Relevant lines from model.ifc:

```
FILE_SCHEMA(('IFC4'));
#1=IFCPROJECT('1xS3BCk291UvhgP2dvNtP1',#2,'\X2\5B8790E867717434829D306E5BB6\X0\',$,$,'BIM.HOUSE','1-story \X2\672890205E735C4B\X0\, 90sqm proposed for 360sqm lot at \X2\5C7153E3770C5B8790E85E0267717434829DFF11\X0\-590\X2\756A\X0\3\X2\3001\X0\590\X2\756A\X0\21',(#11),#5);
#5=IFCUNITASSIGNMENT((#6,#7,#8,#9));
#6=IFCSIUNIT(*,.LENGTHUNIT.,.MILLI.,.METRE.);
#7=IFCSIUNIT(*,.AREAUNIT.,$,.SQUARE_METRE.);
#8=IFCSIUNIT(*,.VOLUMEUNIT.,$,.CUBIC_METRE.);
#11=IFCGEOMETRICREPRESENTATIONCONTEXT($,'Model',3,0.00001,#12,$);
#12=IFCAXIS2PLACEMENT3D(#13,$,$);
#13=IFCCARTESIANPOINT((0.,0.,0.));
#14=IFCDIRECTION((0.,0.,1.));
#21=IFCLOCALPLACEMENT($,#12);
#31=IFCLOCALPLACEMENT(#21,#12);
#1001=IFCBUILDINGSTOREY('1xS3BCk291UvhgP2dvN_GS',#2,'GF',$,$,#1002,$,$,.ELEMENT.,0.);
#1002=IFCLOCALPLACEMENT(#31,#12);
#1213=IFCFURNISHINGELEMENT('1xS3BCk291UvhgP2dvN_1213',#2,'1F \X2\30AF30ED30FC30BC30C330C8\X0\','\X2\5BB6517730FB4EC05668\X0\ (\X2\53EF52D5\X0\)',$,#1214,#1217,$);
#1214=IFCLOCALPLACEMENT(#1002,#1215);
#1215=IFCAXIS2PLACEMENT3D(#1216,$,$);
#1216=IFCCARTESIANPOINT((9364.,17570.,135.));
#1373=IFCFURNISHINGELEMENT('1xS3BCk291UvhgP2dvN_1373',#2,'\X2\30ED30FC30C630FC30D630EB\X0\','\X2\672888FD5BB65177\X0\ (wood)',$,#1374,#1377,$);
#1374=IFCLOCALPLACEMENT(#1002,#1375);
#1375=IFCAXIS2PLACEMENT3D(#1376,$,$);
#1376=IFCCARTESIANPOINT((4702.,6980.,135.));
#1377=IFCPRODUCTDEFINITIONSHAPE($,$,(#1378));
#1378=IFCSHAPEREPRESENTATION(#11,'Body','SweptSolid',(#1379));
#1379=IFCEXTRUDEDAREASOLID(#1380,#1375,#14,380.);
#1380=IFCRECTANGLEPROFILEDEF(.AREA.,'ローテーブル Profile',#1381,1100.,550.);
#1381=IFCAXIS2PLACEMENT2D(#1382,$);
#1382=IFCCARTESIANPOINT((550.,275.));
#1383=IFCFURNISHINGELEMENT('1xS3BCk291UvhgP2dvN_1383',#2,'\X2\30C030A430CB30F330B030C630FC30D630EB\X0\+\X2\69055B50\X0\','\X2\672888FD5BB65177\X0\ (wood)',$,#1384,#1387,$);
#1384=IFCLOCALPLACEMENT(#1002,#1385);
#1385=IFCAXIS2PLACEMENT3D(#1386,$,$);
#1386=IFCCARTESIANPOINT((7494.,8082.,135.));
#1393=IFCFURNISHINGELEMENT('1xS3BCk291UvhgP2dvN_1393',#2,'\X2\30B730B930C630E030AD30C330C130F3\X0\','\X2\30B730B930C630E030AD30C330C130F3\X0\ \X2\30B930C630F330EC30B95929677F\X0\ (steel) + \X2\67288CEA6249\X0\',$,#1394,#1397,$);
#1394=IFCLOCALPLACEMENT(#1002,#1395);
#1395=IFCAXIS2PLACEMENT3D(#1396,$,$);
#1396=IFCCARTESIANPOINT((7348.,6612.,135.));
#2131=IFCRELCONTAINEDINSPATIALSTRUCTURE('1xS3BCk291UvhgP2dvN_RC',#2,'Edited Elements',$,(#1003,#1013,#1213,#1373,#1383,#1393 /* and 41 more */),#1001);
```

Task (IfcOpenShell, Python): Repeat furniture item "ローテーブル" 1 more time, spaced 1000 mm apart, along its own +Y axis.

```python
import ifcopenshell
import ifcopenshell.api.geometry
import ifcopenshell.api.root
import ifcopenshell.util.element
import ifcopenshell.util.placement
import ifcopenshell.util.unit

model = ifcopenshell.open("model.ifc")
unit_scale = ifcopenshell.util.unit.calculate_unit_scale(model)


def reuse_history(source, copy):
    """copy_class also copies each property set's owner history, people and application; keep the originals."""
    for rel in copy.IsDefinedBy:
        if rel.is_a("IfcRelDefinesByProperties") and (history := rel.RelatingPropertyDefinition.OwnerHistory):
            rel.RelatingPropertyDefinition.OwnerHistory = source.OwnerHistory
            ifcopenshell.util.element.remove_deep2(model, history)


source = model.by_guid("1xS3BCk291UvhgP2dvN_1373")
base = ifcopenshell.util.placement.get_local_placement(source.ObjectPlacement)
step = base[:3, 1] * 1 / unit_scale

for i in range(1, 2):
    copy = ifcopenshell.api.root.copy_class(model, product=source)
    copy.Representation = ifcopenshell.util.element.copy_deep(
        model, source.Representation, exclude=["IfcGeometricRepresentationContext", "IfcRepresentationMap"]
    )
    reuse_history(source, copy)
    matrix = base.copy()
    matrix[:3, 3] += i * step
    print("added at", matrix[:3, 3].round(3) + 0.0)
    ifcopenshell.api.geometry.edit_object_placement(model, product=copy, matrix=matrix, is_si=False)

model.write("model_edited.ifc")
```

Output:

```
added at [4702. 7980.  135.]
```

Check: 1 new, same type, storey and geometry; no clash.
